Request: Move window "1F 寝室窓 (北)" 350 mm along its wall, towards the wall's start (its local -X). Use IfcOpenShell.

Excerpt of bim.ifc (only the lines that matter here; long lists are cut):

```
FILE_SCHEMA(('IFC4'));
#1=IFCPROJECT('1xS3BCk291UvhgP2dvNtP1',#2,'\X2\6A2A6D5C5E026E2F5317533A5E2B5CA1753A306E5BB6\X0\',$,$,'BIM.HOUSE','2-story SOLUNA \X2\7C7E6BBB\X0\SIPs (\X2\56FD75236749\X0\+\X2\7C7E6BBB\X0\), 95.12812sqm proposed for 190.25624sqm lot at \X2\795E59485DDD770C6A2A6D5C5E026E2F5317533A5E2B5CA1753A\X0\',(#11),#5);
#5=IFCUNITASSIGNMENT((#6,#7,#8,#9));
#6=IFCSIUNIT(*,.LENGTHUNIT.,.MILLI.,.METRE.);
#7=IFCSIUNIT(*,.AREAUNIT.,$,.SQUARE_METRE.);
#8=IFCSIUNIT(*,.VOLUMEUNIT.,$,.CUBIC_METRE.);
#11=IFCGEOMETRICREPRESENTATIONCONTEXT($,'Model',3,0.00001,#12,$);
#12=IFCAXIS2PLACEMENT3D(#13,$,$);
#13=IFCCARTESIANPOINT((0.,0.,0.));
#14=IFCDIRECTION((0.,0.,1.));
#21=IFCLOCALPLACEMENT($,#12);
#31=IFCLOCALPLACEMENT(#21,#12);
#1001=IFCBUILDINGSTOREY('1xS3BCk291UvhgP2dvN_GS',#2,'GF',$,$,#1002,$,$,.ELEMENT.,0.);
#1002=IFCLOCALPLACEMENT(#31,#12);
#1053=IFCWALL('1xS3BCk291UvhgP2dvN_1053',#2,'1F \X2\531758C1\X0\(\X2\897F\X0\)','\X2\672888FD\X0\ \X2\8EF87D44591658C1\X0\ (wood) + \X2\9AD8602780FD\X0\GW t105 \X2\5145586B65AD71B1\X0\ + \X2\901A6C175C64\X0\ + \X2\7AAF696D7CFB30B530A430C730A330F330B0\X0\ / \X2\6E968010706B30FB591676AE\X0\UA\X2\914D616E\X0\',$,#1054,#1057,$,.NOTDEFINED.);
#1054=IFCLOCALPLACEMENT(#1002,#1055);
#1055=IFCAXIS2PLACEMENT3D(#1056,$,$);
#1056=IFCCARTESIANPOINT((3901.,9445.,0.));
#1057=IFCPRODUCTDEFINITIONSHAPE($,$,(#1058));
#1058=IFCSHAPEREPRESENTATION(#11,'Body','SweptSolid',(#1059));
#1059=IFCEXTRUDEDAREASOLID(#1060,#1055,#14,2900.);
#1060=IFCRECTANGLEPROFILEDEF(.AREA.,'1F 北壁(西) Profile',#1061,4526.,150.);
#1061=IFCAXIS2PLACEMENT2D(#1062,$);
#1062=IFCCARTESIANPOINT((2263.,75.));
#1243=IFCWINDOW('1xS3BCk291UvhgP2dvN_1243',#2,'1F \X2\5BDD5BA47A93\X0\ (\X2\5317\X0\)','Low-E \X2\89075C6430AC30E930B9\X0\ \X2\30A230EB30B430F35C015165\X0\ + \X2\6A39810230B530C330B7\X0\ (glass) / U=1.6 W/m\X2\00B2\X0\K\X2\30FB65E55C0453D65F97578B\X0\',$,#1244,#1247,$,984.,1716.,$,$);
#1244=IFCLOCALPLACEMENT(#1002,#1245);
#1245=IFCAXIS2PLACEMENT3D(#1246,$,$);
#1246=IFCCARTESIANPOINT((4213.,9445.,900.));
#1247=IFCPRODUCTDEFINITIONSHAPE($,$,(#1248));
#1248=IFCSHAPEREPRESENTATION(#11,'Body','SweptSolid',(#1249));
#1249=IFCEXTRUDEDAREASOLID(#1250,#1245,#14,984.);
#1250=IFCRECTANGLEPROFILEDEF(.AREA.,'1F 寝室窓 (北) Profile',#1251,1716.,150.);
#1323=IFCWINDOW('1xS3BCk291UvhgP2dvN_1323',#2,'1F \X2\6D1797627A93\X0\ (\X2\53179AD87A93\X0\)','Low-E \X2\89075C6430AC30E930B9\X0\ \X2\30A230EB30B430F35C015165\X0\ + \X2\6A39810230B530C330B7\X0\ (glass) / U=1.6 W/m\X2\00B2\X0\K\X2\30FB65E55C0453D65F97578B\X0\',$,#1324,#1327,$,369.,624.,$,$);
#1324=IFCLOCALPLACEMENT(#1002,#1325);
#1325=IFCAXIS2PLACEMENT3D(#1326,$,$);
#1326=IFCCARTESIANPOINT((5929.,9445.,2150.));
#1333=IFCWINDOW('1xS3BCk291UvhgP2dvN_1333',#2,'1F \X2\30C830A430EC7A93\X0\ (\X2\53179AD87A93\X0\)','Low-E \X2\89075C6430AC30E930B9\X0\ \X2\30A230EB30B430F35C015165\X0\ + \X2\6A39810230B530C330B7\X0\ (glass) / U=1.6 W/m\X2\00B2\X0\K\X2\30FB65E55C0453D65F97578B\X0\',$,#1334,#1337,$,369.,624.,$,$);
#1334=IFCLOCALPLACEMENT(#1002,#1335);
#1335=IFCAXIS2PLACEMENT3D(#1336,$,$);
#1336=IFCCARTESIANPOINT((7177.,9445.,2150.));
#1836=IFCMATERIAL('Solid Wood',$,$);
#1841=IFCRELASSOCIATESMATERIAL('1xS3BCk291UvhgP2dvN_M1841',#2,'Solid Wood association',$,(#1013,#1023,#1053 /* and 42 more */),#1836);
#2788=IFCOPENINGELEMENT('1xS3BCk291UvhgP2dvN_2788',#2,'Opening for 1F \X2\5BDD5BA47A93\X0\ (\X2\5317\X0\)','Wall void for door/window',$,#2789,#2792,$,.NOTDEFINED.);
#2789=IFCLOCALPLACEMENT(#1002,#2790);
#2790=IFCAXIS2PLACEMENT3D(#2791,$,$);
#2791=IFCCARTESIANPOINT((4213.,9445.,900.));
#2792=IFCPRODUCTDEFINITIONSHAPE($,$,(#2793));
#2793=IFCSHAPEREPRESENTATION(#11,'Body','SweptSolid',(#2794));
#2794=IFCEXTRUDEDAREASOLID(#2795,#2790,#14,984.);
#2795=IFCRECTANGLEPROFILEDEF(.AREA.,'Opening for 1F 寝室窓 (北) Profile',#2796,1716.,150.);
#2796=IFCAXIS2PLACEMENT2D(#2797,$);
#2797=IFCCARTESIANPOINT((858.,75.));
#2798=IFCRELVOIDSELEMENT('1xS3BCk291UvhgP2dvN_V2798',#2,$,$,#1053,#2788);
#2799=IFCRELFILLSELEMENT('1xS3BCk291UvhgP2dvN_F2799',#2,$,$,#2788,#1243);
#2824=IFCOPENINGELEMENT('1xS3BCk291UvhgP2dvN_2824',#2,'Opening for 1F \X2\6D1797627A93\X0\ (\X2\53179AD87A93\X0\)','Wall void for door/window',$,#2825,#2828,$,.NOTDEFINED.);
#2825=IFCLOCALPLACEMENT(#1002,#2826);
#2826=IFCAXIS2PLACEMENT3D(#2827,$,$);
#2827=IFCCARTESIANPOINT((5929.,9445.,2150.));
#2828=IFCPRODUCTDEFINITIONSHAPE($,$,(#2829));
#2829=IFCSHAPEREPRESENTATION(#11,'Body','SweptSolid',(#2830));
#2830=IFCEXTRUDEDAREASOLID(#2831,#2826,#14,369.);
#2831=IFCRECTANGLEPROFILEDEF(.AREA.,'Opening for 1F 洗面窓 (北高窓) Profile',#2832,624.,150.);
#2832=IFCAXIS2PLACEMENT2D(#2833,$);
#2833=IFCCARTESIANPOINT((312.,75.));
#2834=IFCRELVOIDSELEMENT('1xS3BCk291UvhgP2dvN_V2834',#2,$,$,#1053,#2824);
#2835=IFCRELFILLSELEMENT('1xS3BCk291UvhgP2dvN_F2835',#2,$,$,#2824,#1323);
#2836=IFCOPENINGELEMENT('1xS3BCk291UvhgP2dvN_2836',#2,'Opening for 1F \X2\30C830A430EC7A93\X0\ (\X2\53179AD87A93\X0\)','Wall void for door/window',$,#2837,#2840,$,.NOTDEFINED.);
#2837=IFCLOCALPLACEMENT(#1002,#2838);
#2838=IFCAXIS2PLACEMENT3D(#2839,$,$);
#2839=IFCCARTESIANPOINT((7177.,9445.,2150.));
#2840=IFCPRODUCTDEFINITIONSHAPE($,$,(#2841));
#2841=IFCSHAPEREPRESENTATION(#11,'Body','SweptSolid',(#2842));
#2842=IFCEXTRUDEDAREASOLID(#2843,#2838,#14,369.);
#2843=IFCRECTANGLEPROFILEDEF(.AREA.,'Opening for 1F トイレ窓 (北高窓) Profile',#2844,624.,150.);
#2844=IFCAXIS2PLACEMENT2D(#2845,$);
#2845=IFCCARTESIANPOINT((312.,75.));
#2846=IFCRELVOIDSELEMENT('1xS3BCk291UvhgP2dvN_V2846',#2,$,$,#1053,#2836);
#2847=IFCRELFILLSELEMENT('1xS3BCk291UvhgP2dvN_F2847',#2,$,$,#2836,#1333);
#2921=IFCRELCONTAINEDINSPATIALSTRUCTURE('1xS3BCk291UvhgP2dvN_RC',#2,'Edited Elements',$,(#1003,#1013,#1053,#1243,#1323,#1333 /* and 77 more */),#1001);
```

```python
import ifcopenshell
import ifcopenshell.api.geometry
import ifcopenshell.util.placement
import ifcopenshell.util.unit

model = ifcopenshell.open("bim.ifc")
unit_scale = ifcopenshell.util.unit.calculate_unit_scale(model)

window = model.by_guid("1xS3BCk291UvhgP2dvN_1243")
opening = window.FillsVoids[0].RelatingOpeningElement
wall = opening.VoidsElements[0].RelatingBuildingElement

wall_matrix = ifcopenshell.util.placement.get_local_placement(wall.ObjectPlacement)
shift = wall_matrix[:3, 0] * -0.35 / unit_scale
before = ifcopenshell.util.placement.get_local_placement(window.ObjectPlacement)[:3, 3].copy()

# The window is not placed relative to its opening, so move both.
for product in (opening, window):
    matrix = ifcopenshell.util.placement.get_local_placement(product.ObjectPlacement)
    matrix[:3, 3] += shift
    ifcopenshell.api.geometry.edit_object_placement(model, product=product, matrix=matrix, is_si=False)

after = ifcopenshell.util.placement.get_local_placement(window.ObjectPlacement)[:3, 3]
print("window moved by", (after - before).round(3) + 0.0)

model.write("bim_updated.ifc")
```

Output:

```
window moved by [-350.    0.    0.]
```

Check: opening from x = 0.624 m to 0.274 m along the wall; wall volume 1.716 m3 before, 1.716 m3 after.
